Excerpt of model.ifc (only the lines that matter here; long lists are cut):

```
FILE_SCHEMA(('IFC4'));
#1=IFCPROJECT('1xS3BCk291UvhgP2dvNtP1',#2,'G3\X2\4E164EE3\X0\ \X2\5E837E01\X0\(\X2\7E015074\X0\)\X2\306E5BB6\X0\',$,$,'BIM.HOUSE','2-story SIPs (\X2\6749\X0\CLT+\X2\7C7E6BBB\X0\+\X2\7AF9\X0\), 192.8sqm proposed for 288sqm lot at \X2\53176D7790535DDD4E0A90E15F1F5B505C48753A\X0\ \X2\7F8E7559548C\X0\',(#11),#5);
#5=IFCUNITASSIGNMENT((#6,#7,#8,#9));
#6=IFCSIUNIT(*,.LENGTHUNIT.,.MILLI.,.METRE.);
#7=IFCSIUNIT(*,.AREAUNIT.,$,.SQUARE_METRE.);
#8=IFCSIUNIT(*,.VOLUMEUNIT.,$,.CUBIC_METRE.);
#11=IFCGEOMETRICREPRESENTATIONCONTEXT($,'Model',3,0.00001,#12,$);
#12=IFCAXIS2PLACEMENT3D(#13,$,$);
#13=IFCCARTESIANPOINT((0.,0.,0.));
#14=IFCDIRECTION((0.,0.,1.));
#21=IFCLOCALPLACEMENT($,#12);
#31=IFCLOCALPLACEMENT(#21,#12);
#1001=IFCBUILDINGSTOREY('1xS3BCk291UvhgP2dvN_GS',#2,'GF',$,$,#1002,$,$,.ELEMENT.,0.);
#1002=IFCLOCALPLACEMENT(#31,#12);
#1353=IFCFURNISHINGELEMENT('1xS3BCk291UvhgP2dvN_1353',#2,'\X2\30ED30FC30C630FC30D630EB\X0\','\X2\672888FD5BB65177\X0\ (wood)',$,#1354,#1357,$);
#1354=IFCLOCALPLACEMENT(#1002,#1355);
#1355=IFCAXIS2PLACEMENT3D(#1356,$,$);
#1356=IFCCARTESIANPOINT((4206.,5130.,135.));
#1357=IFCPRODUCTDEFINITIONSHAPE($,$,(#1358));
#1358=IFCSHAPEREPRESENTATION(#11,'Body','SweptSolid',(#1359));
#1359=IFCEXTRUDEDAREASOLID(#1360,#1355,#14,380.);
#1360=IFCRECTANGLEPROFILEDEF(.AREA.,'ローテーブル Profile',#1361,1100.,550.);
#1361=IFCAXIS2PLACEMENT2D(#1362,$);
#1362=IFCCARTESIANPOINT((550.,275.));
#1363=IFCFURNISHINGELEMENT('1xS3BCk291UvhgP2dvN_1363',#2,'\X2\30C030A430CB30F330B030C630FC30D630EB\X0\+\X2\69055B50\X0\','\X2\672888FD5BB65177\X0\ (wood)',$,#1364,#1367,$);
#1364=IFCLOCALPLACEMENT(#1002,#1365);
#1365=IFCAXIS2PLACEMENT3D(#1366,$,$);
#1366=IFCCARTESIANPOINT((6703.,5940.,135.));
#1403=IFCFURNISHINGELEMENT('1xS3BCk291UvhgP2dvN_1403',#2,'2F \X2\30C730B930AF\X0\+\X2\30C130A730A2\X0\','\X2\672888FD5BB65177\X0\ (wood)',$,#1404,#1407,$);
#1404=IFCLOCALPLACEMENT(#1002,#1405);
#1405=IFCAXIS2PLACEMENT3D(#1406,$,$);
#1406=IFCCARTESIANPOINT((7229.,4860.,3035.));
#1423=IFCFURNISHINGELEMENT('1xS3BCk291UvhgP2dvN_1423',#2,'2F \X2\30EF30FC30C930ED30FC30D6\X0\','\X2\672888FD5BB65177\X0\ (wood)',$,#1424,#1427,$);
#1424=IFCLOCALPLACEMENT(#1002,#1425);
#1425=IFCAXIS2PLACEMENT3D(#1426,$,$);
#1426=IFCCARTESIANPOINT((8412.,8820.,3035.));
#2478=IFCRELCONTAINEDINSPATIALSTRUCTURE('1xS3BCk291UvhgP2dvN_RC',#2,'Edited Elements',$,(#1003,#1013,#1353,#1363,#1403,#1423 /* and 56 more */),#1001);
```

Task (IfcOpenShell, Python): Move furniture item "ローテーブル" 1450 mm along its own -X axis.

```python
import ifcopenshell
import ifcopenshell.api.geometry
import ifcopenshell.util.placement

model = ifcopenshell.open("model.ifc")

item = model.by_guid("1xS3BCk291UvhgP2dvN_1353")
matrix = ifcopenshell.util.placement.get_local_placement(item.ObjectPlacement)
matrix[:3, 3] -= matrix[:3, 0] * 1450.0
ifcopenshell.api.geometry.edit_object_placement(model, product=item, matrix=matrix, is_si=False)

print(ifcopenshell.util.placement.get_local_placement(item.ObjectPlacement).round(3) + 0.0)

model.write("model_rev.ifc")
```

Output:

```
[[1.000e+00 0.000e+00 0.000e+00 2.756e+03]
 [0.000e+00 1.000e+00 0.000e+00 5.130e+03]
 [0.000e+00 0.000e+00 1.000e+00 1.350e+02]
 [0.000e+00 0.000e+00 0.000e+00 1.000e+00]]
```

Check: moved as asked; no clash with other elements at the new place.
